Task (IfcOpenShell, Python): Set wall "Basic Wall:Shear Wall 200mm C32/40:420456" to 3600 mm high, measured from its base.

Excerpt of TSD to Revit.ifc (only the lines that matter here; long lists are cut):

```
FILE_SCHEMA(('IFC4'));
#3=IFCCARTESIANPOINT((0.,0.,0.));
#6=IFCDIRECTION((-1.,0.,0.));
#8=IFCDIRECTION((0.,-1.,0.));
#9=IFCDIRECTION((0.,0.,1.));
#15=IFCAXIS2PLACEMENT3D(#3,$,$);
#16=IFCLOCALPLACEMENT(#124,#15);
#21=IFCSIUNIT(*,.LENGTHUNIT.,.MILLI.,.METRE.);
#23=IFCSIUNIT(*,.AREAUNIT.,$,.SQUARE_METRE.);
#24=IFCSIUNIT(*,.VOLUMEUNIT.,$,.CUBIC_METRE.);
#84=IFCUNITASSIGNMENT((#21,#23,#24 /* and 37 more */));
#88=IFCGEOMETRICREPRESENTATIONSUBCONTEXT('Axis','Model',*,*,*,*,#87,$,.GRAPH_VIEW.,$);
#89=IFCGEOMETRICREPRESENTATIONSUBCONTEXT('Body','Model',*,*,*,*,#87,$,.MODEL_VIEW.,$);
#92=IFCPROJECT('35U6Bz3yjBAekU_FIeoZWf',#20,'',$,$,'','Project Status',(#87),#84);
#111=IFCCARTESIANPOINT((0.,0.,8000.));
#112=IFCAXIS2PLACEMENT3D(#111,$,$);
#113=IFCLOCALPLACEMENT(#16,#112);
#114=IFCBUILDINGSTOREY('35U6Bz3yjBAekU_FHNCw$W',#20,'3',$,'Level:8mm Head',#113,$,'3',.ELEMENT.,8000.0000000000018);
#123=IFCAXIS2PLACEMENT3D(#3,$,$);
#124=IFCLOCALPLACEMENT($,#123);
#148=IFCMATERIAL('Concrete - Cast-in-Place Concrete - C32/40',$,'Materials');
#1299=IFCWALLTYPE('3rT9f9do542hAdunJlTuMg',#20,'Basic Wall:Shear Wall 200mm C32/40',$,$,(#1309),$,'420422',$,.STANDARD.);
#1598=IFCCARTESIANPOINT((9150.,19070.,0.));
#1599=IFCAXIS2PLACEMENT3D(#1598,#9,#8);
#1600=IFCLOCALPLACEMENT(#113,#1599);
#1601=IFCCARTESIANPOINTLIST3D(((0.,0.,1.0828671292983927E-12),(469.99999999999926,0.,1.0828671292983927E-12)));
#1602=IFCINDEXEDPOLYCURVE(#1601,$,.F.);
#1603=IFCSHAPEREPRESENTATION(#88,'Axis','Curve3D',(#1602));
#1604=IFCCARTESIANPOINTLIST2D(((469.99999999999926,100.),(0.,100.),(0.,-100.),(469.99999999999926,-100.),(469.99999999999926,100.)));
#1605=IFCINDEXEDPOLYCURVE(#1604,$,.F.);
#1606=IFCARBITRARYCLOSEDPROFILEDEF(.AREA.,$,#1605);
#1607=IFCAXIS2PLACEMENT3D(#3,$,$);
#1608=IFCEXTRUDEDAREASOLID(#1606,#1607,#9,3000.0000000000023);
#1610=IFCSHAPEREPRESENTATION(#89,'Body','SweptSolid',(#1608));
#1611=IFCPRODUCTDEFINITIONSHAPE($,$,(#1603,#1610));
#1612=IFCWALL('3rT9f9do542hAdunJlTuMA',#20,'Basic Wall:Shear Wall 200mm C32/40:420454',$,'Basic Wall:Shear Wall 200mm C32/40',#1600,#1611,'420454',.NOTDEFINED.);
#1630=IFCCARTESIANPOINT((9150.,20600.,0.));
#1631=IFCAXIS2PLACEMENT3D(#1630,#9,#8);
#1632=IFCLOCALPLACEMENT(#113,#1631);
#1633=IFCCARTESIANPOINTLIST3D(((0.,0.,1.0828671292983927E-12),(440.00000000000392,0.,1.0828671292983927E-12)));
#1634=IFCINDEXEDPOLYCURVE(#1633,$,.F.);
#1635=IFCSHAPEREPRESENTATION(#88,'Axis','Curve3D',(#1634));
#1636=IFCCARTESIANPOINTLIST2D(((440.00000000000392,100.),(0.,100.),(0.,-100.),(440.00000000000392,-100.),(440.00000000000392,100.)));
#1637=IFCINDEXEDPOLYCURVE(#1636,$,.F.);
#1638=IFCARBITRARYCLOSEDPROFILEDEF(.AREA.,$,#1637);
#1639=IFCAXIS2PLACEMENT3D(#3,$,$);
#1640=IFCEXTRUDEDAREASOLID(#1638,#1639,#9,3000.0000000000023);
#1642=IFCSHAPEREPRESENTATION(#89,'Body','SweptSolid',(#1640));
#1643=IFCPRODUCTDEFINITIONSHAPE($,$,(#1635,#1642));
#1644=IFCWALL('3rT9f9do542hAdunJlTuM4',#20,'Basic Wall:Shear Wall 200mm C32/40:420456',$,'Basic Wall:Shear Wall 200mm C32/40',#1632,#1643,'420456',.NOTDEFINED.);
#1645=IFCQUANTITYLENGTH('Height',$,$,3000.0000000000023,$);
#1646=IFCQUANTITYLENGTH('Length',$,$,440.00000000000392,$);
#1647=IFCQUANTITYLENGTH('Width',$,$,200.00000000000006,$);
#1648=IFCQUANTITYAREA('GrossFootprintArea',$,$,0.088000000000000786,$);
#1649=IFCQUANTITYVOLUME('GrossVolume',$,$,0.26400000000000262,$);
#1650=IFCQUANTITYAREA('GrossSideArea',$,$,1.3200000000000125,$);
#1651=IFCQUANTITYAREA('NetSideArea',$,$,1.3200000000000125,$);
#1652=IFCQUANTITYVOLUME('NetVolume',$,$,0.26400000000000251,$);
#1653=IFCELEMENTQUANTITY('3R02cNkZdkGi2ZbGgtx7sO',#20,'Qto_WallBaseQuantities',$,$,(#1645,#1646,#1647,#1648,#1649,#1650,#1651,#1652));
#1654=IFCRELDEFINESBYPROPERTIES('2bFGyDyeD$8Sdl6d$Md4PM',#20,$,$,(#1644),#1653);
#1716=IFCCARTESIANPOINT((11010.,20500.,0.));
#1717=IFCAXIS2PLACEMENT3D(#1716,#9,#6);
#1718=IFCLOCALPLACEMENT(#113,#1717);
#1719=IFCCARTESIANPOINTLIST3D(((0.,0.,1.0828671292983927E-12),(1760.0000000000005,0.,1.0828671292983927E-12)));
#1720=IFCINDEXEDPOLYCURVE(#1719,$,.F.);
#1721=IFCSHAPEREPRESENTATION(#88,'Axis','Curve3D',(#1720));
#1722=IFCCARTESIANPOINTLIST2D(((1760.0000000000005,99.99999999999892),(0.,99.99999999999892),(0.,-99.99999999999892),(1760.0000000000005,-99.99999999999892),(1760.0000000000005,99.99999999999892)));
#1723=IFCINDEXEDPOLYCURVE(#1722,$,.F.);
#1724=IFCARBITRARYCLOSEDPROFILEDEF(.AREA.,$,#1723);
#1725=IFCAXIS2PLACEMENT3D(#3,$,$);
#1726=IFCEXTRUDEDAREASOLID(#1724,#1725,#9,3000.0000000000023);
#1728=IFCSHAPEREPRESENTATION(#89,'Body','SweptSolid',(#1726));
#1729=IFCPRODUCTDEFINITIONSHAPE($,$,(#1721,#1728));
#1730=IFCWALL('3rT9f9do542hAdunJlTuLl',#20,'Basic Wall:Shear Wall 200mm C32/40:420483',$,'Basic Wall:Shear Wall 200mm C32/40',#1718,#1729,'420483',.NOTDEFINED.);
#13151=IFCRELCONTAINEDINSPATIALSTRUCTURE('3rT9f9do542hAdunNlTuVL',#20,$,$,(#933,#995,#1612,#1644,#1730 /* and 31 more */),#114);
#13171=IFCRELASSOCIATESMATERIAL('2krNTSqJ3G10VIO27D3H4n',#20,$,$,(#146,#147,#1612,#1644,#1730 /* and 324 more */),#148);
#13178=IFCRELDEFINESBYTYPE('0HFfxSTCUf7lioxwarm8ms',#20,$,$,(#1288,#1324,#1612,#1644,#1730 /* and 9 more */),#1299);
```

```python
import ifcopenshell
import ifcopenshell.api.pset
import ifcopenshell.geom
import ifcopenshell.util.element
import ifcopenshell.util.representation
import ifcopenshell.util.shape
import ifcopenshell.util.unit

model = ifcopenshell.open("TSD to Revit.ifc")
unit_scale = ifcopenshell.util.unit.calculate_unit_scale(model)
area_scale = ifcopenshell.util.unit.calculate_unit_scale(model, "AREAUNIT")
volume_scale = ifcopenshell.util.unit.calculate_unit_scale(model, "VOLUMEUNIT")
settings = ifcopenshell.geom.settings()


def volume(element):
    """Net volume in cubic metres, openings subtracted."""
    shape = ifcopenshell.geom.create_shape(settings, element)
    return ifcopenshell.util.shape.get_volume(shape.geometry)


wall = model.by_guid("3rT9f9do542hAdunJlTuM4")
before = volume(wall)

body = ifcopenshell.util.representation.get_representation(wall, "Model", "Body")
solid = body.Items[0]
old_height = solid.Depth
solid.Depth = 3600.0
after = volume(wall)
thickness = 0.2  # wall thickness in metres

# Update the stored height, areas and volumes.
qto = model.by_id(ifcopenshell.util.element.get_pset(wall, "Qto_WallBaseQuantities", should_inherit=False)["id"])
ifcopenshell.api.pset.edit_qto(model, qto=qto, properties={
    "Height": solid.Depth,
    "GrossVolume": ifcopenshell.util.element.get_pset(wall, "Qto_WallBaseQuantities", "GrossVolume") * solid.Depth / old_height,
    "GrossSideArea": ifcopenshell.util.element.get_pset(wall, "Qto_WallBaseQuantities", "GrossSideArea") * solid.Depth / old_height,
    "NetSideArea": after / thickness / area_scale,
    "NetVolume": after / volume_scale,
})

print(f"height {old_height:g} -> {solid.Depth:g}, volume {before:.3f} -> {after:.3f} m3")

model.write("TSD to Revit_rev.ifc")
```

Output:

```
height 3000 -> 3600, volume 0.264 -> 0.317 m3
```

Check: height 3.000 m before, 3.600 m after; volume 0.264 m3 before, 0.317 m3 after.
